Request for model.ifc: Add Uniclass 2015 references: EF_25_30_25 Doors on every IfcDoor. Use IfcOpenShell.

First a look at what the model holds.

```python
import ifcopenshell

model = ifcopenshell.open("model.ifc")
print(model.schema)
print("classifications:", [c.Name for c in model.by_type("IfcClassification")])
for ifc_class in ("IfcDoor", "IfcRoof", "IfcStair", "IfcWall", "IfcWindow"):
    print(ifc_class, len(model.by_type(ifc_class)))
```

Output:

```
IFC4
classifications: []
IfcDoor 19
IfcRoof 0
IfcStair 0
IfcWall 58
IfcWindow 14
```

```python
import ifcopenshell
import ifcopenshell.api.classification

model = ifcopenshell.open("model.ifc")

system = ifcopenshell.api.classification.add_classification(model, classification="Uniclass 2015")

codes = {
    "IfcDoor": ("EF_25_30_25", "Doors"),
}
for ifc_class, (code, name) in codes.items():
    products = model.by_type(ifc_class)
    ifcopenshell.api.classification.add_reference(
        model, products=products, classification=system, identification=code, name=name
    )
    print(code, len(products))

model.write("model_updated.ifc")
```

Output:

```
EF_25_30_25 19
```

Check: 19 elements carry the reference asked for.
